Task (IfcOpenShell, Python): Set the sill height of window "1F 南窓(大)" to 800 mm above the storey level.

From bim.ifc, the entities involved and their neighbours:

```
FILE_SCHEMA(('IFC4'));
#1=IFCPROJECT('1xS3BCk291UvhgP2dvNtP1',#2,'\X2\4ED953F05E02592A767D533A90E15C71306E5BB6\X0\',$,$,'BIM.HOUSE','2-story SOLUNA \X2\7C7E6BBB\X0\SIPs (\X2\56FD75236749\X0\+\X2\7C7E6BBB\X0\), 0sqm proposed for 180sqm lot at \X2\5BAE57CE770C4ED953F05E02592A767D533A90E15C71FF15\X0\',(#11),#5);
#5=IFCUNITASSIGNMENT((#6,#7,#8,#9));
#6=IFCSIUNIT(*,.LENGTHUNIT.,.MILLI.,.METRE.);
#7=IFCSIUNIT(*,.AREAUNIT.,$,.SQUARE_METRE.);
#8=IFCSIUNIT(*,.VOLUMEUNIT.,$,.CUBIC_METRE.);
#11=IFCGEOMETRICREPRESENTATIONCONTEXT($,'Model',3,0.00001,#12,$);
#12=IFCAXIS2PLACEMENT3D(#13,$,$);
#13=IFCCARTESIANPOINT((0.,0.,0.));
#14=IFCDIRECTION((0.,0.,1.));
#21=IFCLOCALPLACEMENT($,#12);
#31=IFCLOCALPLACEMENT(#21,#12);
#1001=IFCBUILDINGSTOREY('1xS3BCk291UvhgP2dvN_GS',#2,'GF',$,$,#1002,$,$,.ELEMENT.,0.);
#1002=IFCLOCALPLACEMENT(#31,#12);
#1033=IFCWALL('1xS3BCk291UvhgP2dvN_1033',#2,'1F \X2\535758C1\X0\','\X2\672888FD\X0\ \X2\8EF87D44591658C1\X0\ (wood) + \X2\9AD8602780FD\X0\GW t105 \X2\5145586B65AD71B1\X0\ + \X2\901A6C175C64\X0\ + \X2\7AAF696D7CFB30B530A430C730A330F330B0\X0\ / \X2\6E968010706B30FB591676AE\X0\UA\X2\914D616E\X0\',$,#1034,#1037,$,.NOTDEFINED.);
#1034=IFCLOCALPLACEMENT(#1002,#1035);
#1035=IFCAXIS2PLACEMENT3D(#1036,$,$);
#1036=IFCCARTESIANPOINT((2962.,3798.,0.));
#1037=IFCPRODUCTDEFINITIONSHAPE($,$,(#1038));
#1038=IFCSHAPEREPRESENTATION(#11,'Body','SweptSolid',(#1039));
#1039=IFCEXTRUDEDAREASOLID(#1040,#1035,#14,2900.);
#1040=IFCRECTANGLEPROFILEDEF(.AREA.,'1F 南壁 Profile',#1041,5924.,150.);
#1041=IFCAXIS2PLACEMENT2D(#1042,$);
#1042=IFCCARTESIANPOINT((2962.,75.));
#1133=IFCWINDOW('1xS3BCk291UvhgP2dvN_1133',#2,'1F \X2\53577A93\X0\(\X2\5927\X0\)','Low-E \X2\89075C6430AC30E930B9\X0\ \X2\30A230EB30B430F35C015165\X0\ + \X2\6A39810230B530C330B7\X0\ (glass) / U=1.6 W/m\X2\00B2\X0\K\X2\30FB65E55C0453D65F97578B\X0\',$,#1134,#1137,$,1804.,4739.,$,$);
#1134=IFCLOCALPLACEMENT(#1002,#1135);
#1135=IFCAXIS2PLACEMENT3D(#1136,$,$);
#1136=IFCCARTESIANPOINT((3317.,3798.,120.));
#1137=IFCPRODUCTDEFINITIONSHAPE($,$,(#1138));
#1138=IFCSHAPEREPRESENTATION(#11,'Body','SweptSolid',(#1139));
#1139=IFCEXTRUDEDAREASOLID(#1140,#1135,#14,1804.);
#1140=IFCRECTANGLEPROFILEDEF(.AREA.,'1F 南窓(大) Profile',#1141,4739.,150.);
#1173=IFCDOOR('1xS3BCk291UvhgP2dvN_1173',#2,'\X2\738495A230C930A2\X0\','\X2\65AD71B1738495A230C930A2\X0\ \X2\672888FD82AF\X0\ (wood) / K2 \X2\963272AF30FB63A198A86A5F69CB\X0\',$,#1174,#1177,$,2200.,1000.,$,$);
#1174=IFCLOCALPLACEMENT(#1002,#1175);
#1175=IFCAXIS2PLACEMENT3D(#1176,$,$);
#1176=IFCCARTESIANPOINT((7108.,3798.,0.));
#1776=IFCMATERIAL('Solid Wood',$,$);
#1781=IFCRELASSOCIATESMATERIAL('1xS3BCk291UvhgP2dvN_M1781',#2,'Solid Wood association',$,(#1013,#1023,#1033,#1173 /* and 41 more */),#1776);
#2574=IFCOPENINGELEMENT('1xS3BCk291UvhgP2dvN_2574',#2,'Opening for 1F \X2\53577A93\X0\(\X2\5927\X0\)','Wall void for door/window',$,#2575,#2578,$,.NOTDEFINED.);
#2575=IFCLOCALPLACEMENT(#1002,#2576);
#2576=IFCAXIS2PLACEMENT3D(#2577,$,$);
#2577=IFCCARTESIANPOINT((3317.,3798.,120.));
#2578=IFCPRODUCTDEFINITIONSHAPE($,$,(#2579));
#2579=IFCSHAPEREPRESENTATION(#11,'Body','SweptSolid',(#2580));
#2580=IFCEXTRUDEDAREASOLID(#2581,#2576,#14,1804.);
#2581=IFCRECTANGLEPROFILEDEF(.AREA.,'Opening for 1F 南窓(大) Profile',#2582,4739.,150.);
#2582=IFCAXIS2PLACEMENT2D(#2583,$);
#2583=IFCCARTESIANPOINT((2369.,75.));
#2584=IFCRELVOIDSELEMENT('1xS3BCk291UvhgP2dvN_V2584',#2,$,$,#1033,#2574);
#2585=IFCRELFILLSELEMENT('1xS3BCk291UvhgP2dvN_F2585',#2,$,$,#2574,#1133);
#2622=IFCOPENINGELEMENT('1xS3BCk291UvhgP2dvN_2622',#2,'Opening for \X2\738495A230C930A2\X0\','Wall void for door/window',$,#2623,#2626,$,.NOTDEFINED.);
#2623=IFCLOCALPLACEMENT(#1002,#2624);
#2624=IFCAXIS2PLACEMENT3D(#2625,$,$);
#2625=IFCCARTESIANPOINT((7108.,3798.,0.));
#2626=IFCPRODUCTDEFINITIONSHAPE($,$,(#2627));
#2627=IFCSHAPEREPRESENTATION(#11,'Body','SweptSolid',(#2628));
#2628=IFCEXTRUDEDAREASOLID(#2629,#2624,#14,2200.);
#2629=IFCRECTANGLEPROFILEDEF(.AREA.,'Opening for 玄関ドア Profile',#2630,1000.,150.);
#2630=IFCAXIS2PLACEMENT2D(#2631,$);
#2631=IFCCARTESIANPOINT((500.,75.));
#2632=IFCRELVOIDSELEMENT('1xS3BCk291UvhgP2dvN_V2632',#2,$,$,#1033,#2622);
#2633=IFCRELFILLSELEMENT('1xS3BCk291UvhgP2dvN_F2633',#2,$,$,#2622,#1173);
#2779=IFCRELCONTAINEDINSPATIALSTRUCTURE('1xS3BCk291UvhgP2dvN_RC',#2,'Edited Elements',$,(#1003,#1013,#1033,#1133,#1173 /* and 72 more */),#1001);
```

```python
import numpy as np
import ifcopenshell
import ifcopenshell.api.geometry
import ifcopenshell.geom
import ifcopenshell.util.element
import ifcopenshell.util.placement
import ifcopenshell.util.shape
import ifcopenshell.util.unit

model = ifcopenshell.open("bim.ifc")
unit_scale = ifcopenshell.util.unit.calculate_unit_scale(model)

window = model.by_guid("1xS3BCk291UvhgP2dvN_1133")
opening = window.FillsVoids[0].RelatingOpeningElement
storey = ifcopenshell.util.element.get_container(window, ifc_class="IfcBuildingStorey")
level = ifcopenshell.util.placement.get_local_placement(storey.ObjectPlacement)[2, 3]

# The opening's origin need not be at the sill, so measure its lowest point.
shape = ifcopenshell.geom.create_shape(ifcopenshell.geom.settings(), opening)
bottom = ifcopenshell.util.shape.get_shape_bottom_elevation(shape, shape.geometry) / unit_scale
dz = level + 0.8 / unit_scale - bottom

shift = np.array([0.0, 0.0, dz])
# The window is not placed relative to its opening, so move both.
for product in (opening, window):
    matrix = ifcopenshell.util.placement.get_local_placement(product.ObjectPlacement)
    matrix[:3, 3] += shift
    ifcopenshell.api.geometry.edit_object_placement(model, product=product, matrix=matrix, is_si=False)

print(f"moved by {dz * unit_scale:+.3f} m")

model.write("bim-out.ifc")
```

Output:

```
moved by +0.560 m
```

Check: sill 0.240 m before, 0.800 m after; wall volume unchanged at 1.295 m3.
